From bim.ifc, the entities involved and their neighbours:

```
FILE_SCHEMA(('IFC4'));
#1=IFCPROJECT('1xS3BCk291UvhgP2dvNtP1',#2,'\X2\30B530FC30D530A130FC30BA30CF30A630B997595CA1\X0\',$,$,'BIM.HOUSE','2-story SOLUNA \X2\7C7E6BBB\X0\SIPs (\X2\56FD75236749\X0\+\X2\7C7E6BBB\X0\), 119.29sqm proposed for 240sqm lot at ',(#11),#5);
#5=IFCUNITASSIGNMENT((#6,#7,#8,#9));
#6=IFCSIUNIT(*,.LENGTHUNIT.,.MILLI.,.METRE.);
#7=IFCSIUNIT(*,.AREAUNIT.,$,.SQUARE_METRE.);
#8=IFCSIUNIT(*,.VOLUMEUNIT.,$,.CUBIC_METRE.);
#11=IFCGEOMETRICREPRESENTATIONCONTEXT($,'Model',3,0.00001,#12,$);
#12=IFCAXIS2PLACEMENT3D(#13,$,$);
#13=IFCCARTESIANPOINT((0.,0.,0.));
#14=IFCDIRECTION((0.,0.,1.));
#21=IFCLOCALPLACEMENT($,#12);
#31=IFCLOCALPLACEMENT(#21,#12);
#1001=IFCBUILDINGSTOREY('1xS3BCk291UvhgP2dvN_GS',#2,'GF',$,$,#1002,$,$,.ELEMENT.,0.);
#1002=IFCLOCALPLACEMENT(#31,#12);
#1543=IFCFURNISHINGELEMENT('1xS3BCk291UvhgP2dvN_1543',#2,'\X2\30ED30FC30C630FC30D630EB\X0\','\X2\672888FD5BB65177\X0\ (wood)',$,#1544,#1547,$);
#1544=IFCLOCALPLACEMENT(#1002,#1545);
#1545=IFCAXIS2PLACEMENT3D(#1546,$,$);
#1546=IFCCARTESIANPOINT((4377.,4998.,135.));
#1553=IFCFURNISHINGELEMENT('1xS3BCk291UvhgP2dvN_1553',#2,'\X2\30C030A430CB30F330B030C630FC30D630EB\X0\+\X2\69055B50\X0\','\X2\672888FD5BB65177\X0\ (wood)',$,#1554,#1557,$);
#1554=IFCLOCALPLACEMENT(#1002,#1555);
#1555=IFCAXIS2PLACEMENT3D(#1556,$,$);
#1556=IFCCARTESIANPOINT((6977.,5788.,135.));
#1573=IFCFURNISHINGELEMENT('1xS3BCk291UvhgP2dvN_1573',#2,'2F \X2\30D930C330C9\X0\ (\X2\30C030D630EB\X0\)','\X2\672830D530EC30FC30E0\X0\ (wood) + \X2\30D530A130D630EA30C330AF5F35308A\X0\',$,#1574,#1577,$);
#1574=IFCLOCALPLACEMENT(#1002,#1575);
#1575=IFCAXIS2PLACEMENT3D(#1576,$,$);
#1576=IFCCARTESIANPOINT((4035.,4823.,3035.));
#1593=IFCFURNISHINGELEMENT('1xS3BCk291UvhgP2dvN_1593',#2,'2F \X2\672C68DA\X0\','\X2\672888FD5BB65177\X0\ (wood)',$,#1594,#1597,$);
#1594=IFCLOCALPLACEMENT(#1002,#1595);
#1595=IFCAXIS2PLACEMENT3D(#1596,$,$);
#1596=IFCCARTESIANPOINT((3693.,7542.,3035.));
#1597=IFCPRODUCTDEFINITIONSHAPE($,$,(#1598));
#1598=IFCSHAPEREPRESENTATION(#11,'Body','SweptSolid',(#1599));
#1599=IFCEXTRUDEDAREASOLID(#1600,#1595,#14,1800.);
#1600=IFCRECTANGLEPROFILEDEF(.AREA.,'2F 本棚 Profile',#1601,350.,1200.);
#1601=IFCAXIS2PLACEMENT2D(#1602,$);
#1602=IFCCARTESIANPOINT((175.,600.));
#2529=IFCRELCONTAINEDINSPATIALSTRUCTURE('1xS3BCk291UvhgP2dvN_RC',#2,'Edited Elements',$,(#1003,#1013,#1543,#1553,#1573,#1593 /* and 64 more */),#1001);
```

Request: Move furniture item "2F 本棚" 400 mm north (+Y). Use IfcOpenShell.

```python
import ifcopenshell
import ifcopenshell.api.geometry
import ifcopenshell.util.placement
import ifcopenshell.util.unit

model = ifcopenshell.open("bim.ifc")
unit_scale = ifcopenshell.util.unit.calculate_unit_scale(model)

item = model.by_guid("1xS3BCk291UvhgP2dvN_1593")
matrix = ifcopenshell.util.placement.get_local_placement(item.ObjectPlacement)
matrix[1, 3] += 0.4 / unit_scale
ifcopenshell.api.geometry.edit_object_placement(model, product=item, matrix=matrix, is_si=False)

print(ifcopenshell.util.placement.get_local_placement(item.ObjectPlacement).round(3) + 0.0)

model.write("bim-out.ifc")
```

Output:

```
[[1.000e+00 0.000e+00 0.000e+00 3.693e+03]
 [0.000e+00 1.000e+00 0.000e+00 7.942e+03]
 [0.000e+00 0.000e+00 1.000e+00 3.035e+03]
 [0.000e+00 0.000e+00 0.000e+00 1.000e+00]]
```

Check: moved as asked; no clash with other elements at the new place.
